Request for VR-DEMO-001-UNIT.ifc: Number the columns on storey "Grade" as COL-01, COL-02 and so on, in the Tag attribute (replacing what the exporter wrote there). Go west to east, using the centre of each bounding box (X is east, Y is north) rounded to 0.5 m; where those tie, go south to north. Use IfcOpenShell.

First a look at what the model holds.

```python
import ifcopenshell
import ifcopenshell.util.element
import ifcopenshell.util.placement

model = ifcopenshell.open("VR-DEMO-001-UNIT.ifc")
print(model.schema)
storey = next(s for s in model.by_type("IfcBuildingStorey") if s.Name == "Grade")
columns = [e for e in ifcopenshell.util.element.get_decomposition(storey) if e.is_a("IfcColumn")]
for e in sorted(columns, key=lambda e: e.id()):
    origin = ifcopenshell.util.placement.get_local_placement(e.ObjectPlacement)[:3, 3]
    print(e.id(), e.Tag, e.Name, origin.round(2) + 0.0, sep=" | ")
```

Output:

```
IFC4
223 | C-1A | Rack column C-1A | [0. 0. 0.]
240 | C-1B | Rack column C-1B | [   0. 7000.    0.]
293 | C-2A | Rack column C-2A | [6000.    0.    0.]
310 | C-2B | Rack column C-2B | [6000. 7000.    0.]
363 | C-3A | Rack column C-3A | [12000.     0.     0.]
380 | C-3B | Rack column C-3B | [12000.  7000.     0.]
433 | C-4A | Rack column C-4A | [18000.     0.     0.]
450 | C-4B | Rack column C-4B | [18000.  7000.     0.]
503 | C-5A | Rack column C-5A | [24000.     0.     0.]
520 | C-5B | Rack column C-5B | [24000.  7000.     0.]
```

```python
import ifcopenshell
import ifcopenshell.geom
import ifcopenshell.util.element
import ifcopenshell.util.shape

model = ifcopenshell.open("VR-DEMO-001-UNIT.ifc")
settings = ifcopenshell.geom.settings()
settings.set("use-world-coords", True)


def centre(element):
    shape = ifcopenshell.geom.create_shape(settings, element)
    return ifcopenshell.util.shape.get_bbox_centroid(shape.geometry)


storey = next(s for s in model.by_type("IfcBuildingStorey") if s.Name == "Grade")
columns = [e for e in ifcopenshell.util.element.get_decomposition(storey) if e.is_a("IfcColumn")]

# Insertion points can sit at a corner or the storey origin, so sort by the geometry (in metres).
centres = {e: centre(e) for e in columns}
columns.sort(key=lambda e: (round(centres[e][0] / 0.5), centres[e][1]))

for i, e in enumerate(columns, start=1):
    number = f"COL-{i:02d}"
    e.Tag = number
    print(e.id(), number)

model.write("VR-DEMO-001-UNIT-out.ifc")
```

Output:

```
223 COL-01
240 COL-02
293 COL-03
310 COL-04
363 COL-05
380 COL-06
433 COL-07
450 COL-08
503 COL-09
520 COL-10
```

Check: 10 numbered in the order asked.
